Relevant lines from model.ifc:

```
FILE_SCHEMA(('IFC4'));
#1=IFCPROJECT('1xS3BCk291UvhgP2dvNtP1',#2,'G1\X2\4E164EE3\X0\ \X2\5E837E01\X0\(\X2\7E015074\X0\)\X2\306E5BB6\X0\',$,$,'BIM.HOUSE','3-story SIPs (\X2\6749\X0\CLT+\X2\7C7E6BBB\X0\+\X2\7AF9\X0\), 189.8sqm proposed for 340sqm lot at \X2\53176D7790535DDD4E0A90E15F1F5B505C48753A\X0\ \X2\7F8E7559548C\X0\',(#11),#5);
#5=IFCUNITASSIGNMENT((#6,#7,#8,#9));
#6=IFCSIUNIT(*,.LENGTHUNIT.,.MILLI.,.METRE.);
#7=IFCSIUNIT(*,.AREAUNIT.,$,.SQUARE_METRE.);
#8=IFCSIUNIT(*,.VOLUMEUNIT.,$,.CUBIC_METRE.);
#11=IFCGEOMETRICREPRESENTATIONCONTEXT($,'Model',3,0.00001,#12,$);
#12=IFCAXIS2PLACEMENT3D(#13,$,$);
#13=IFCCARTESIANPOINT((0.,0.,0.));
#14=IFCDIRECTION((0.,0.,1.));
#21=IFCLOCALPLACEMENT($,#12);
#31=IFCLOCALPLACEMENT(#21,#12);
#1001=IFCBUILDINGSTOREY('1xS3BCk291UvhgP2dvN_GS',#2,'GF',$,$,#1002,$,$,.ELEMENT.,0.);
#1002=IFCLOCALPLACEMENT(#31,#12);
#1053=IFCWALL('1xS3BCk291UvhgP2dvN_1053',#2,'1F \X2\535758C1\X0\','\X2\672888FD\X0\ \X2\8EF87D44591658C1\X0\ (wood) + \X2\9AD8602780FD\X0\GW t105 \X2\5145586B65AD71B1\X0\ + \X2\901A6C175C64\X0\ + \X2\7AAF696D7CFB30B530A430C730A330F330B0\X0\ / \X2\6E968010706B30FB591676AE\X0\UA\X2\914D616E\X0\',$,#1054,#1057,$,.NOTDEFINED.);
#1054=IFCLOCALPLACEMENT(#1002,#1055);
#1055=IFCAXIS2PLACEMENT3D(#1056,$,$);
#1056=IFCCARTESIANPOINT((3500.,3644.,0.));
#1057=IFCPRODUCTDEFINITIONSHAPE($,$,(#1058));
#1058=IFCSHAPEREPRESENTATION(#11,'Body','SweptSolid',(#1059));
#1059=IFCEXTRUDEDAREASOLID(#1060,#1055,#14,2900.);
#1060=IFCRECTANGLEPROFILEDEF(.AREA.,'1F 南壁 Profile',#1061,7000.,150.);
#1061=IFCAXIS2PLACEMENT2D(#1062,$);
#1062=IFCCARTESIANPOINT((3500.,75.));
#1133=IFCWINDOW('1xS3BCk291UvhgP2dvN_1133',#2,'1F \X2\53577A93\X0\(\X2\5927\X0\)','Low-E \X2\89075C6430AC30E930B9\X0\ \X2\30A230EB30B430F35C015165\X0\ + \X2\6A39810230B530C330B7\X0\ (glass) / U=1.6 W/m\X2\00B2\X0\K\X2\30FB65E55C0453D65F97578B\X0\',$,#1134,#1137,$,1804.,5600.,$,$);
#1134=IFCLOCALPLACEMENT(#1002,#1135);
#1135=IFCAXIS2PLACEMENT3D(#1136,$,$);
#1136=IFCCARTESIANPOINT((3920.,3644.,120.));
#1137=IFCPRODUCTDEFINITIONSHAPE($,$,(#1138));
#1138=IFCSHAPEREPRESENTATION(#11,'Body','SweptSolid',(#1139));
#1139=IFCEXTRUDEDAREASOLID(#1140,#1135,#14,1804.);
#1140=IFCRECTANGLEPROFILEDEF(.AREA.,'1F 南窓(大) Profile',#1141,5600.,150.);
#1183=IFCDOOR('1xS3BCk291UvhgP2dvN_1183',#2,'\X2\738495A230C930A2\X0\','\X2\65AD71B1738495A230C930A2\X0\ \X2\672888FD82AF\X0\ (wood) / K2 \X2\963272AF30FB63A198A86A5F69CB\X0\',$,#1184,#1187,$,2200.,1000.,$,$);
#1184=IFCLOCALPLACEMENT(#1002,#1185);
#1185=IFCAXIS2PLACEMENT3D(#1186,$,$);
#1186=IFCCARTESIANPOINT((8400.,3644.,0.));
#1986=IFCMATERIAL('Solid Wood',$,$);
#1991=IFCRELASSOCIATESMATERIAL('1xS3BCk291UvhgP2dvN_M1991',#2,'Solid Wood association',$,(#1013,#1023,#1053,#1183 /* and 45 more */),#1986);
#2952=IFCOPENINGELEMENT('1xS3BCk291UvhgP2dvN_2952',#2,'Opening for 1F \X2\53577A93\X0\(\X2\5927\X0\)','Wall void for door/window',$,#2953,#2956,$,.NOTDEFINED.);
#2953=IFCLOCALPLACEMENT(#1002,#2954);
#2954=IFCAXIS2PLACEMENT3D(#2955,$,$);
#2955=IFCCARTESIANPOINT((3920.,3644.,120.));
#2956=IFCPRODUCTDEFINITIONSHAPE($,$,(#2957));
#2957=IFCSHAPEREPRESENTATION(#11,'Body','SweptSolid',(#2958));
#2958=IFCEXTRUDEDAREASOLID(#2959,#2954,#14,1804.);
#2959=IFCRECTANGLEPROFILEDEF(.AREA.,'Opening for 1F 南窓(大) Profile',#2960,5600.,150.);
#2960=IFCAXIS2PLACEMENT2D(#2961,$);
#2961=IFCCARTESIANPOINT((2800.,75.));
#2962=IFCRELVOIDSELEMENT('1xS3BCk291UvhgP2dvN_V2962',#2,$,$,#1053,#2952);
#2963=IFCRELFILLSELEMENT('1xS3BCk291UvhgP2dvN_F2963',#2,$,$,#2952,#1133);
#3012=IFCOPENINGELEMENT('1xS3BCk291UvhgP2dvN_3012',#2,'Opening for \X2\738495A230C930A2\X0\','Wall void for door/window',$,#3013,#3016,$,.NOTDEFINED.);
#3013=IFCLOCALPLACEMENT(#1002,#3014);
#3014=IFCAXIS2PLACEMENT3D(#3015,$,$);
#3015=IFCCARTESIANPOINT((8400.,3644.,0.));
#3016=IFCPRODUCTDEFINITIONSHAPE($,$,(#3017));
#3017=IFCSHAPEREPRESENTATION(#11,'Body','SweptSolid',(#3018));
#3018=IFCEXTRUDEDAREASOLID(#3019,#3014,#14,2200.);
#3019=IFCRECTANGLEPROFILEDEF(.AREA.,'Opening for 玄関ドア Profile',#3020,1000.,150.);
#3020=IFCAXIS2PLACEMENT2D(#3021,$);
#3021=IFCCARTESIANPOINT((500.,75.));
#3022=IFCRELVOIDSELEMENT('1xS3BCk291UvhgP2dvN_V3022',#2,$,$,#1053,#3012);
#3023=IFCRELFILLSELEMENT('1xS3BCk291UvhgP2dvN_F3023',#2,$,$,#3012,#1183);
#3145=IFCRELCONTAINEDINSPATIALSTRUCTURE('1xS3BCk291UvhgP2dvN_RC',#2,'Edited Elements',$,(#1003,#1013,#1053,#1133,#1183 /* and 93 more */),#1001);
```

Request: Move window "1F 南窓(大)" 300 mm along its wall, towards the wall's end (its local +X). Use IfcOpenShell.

```python
import ifcopenshell
import ifcopenshell.api.geometry
import ifcopenshell.util.placement
import ifcopenshell.util.unit

model = ifcopenshell.open("model.ifc")
unit_scale = ifcopenshell.util.unit.calculate_unit_scale(model)

window = model.by_id(1133)
opening = window.FillsVoids[0].RelatingOpeningElement
wall = opening.VoidsElements[0].RelatingBuildingElement

wall_matrix = ifcopenshell.util.placement.get_local_placement(wall.ObjectPlacement)
shift = wall_matrix[:3, 0] * 0.3 / unit_scale
before = ifcopenshell.util.placement.get_local_placement(window.ObjectPlacement)[:3, 3].copy()

# The window is not placed relative to its opening, so move both.
for product in (opening, window):
    matrix = ifcopenshell.util.placement.get_local_placement(product.ObjectPlacement)
    matrix[:3, 3] += shift
    ifcopenshell.api.geometry.edit_object_placement(model, product=product, matrix=matrix, is_si=False)

after = ifcopenshell.util.placement.get_local_placement(window.ObjectPlacement)[:3, 3]
print("window moved by", (after - before).round(3) + 0.0)

model.write("model-out.ifc")
```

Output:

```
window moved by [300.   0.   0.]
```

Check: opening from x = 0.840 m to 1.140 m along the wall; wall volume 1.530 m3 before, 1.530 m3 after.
